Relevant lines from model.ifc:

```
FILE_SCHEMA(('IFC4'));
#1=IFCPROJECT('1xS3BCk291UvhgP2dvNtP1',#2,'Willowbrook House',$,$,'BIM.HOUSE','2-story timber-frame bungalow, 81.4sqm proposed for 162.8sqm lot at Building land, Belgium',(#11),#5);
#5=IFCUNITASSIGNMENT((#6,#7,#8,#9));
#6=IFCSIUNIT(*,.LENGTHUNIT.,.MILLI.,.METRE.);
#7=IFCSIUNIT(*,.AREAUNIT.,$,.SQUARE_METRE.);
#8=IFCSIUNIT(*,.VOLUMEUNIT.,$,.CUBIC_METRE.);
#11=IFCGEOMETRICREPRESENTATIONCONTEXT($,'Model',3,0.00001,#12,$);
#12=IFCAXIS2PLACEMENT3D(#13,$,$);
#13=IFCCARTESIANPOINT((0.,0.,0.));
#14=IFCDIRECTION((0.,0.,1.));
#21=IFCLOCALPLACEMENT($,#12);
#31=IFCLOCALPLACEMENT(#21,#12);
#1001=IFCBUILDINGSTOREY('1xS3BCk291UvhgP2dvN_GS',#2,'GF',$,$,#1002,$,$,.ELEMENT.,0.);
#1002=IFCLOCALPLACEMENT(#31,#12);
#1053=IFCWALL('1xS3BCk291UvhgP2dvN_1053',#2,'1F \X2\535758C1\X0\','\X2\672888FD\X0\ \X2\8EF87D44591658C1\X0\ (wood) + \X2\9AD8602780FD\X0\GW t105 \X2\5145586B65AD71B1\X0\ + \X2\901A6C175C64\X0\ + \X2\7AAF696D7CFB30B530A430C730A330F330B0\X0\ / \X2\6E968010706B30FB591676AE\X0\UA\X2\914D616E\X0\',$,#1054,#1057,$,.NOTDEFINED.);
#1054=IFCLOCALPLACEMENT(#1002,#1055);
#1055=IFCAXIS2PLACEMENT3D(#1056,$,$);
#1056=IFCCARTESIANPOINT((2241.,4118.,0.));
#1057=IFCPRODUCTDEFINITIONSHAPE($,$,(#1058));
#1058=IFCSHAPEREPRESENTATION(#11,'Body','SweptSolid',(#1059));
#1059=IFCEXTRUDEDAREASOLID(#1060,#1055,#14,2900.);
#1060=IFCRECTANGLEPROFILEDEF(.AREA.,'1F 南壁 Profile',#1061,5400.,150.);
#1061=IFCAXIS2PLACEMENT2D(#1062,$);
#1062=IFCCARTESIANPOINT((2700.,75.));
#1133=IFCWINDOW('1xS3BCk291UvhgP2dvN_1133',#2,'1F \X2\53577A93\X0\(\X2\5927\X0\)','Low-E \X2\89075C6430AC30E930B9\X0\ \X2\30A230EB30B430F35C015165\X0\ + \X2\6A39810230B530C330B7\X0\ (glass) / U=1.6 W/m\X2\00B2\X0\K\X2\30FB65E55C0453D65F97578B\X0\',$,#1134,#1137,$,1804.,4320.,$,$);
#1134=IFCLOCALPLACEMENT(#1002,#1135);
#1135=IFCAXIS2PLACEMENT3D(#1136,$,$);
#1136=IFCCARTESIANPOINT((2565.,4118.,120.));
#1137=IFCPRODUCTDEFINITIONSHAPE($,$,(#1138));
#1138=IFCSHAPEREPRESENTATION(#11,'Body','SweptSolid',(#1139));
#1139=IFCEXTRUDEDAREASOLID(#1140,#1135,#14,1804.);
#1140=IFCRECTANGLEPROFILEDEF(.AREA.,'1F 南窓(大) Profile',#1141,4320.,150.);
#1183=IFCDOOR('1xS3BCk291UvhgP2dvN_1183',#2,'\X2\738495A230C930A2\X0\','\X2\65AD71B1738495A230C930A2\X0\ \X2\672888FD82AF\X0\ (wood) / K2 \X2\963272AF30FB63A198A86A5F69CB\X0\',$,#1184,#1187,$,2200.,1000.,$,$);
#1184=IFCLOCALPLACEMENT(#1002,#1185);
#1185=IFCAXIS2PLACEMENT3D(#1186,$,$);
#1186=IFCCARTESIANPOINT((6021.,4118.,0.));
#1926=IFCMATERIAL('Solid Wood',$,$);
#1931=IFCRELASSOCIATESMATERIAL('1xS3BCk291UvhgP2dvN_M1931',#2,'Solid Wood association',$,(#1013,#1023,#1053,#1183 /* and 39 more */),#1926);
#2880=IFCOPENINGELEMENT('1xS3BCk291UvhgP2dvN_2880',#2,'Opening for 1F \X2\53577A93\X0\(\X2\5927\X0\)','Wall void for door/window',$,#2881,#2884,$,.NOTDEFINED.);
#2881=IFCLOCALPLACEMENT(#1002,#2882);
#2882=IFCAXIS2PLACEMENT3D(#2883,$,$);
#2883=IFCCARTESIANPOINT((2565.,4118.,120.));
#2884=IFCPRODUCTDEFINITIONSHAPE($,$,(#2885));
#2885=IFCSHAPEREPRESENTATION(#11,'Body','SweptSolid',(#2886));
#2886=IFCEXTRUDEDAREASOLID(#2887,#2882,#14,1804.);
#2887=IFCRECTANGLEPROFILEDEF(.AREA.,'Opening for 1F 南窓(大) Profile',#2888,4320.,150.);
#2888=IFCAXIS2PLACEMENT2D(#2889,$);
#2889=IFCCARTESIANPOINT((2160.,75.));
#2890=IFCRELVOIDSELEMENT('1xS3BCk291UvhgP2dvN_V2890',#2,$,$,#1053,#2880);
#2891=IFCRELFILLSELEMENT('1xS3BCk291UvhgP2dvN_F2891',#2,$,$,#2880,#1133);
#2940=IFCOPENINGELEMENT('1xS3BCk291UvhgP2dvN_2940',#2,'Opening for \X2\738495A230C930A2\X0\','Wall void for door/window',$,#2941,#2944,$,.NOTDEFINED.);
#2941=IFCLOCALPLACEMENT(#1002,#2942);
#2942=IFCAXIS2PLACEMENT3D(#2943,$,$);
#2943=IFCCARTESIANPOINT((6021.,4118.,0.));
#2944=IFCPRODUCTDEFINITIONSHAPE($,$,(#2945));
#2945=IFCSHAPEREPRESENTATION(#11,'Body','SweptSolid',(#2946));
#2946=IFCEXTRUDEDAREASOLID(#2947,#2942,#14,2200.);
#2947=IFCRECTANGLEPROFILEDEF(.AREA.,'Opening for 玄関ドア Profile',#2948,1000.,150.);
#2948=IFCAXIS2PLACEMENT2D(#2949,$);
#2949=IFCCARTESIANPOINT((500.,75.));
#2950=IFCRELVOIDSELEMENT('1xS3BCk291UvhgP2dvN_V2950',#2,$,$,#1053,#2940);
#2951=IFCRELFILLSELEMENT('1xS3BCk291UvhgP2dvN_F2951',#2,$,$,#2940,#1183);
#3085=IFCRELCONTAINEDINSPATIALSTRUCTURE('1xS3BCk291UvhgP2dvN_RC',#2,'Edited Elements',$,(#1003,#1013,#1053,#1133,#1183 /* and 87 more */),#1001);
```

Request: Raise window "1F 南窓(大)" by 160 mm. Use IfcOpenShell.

```python
import numpy as np
import ifcopenshell
import ifcopenshell.api.geometry
import ifcopenshell.util.placement
import ifcopenshell.util.unit

model = ifcopenshell.open("model.ifc")
unit_scale = ifcopenshell.util.unit.calculate_unit_scale(model)

window = model.by_guid("1xS3BCk291UvhgP2dvN_1133")
opening = window.FillsVoids[0].RelatingOpeningElement
dz = 160.0

shift = np.array([0.0, 0.0, dz])
# The window is not placed relative to its opening, so move both.
for product in (opening, window):
    matrix = ifcopenshell.util.placement.get_local_placement(product.ObjectPlacement)
    matrix[:3, 3] += shift
    ifcopenshell.api.geometry.edit_object_placement(model, product=product, matrix=matrix, is_si=False)

print(f"moved by {dz * unit_scale:+.3f} m")

model.write("model_v2.ifc")
```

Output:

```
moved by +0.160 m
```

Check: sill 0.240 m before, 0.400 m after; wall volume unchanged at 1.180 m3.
